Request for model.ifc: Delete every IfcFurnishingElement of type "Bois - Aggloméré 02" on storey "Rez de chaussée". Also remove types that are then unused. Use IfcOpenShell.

First a look at what the model holds.

```python
import ifcopenshell
import ifcopenshell.util.element

model = ifcopenshell.open("model.ifc")
print(model.schema)
storey = next(s for s in model.by_type("IfcBuildingStorey") if s.Name == "Rez de chaussée")
furniture = [e for e in ifcopenshell.util.element.get_decomposition(storey) if e.is_a("IfcFurnishingElement")]
seen = {}
for e in furniture:
    element_type = ifcopenshell.util.element.get_type(e)
    name = element_type.Name if element_type not in (None, e) else None
    seen[name] = seen.get(name, 0) + 1
for name, count in sorted(seen.items(), key=str):
    print(count, "x", name)
```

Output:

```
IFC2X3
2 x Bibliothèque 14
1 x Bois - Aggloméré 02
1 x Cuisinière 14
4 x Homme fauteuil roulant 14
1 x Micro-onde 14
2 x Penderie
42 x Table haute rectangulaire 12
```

```python
import ifcopenshell
import ifcopenshell.api.root
import ifcopenshell.util.element

model = ifcopenshell.open("model.ifc")

storey = next(s for s in model.by_type("IfcBuildingStorey") if s.Name == "Rez de chaussée")
furniture = [e for e in ifcopenshell.util.element.get_decomposition(storey) if e.is_a("IfcFurnishingElement")]
targets = [e for e in furniture if (t := ifcopenshell.util.element.get_type(e)) not in (None, e) and t.Name == "Bois - Aggloméré 02"]
types = {ifcopenshell.util.element.get_type(e) for e in targets} - {None, *targets}

for e in targets:
    ifcopenshell.api.root.remove_product(model, product=e)
print(len(targets), "removed")

unused = [t for t in types if not ifcopenshell.util.element.get_types(t)]
for t in unused:
    ifcopenshell.api.root.remove_product(model, product=t)
print(len(unused), "unused types removed")

model.write("model_updated.ifc")
```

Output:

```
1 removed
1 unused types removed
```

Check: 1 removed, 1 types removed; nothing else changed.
